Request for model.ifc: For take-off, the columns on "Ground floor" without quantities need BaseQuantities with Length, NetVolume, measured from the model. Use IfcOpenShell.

First a look at what the model holds.

```python
import ifcopenshell
import ifcopenshell.util.element
import ifcopenshell.util.unit

model = ifcopenshell.open("model.ifc")
print(model.schema)
for unit_type in ("LENGTHUNIT", "AREAUNIT", "VOLUMEUNIT"):
    print(unit_type, ifcopenshell.util.unit.calculate_unit_scale(model, unit_type))
storey = next(s for s in model.by_type("IfcBuildingStorey") if s.Name == "Ground floor")
columns = [e for e in ifcopenshell.util.element.get_decomposition(storey) if e.is_a("IfcColumn")]
for e in sorted(columns, key=lambda e: e.id()):
    print(e.id(), e.is_a(), e.Name, list(ifcopenshell.util.element.get_psets(e, qtos_only=True)), sep=" | ")
```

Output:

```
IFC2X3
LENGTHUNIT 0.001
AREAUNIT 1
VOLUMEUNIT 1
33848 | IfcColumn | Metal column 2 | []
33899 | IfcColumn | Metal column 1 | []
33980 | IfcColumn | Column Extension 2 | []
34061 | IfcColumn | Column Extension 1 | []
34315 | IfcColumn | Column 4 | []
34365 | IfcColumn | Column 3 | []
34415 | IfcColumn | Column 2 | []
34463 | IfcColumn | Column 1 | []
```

```python
import ifcopenshell
import ifcopenshell.api.pset
import ifcopenshell.geom
import ifcopenshell.util.element
import ifcopenshell.util.shape
import ifcopenshell.util.unit

model = ifcopenshell.open("model.ifc")
unit_scale = ifcopenshell.util.unit.calculate_unit_scale(model)
volume_scale = ifcopenshell.util.unit.calculate_unit_scale(model, "VOLUMEUNIT")
settings = ifcopenshell.geom.settings()

storey = next(s for s in model.by_type("IfcBuildingStorey") if s.Name == "Ground floor")
columns = [e for e in ifcopenshell.util.element.get_decomposition(storey) if e.is_a("IfcColumn")]

for e in sorted(columns, key=lambda e: e.id()):
    if ifcopenshell.util.element.get_psets(e, qtos_only=True, should_inherit=False):
        continue
    # Geometry comes back in metres, in the element's own axes.
    shape = ifcopenshell.geom.create_shape(settings, e)
    values = {
        "Length": ifcopenshell.util.shape.get_z(shape.geometry) / unit_scale,
        "NetVolume": ifcopenshell.util.shape.get_volume(shape.geometry) / volume_scale,
    }
    qto = ifcopenshell.api.pset.add_qto(model, product=e, name="BaseQuantities")
    ifcopenshell.api.pset.edit_qto(model, qto=qto, properties=values)
    print(e.id(), {k: round(v, 3) for k, v in values.items()})

model.write("model_edited.ifc")
```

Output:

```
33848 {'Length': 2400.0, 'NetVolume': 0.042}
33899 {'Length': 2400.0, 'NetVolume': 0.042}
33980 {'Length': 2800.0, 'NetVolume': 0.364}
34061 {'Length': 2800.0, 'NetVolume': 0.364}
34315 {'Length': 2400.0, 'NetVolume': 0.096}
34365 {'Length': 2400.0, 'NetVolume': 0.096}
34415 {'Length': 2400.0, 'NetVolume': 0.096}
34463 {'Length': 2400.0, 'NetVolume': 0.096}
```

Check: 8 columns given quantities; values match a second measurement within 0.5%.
